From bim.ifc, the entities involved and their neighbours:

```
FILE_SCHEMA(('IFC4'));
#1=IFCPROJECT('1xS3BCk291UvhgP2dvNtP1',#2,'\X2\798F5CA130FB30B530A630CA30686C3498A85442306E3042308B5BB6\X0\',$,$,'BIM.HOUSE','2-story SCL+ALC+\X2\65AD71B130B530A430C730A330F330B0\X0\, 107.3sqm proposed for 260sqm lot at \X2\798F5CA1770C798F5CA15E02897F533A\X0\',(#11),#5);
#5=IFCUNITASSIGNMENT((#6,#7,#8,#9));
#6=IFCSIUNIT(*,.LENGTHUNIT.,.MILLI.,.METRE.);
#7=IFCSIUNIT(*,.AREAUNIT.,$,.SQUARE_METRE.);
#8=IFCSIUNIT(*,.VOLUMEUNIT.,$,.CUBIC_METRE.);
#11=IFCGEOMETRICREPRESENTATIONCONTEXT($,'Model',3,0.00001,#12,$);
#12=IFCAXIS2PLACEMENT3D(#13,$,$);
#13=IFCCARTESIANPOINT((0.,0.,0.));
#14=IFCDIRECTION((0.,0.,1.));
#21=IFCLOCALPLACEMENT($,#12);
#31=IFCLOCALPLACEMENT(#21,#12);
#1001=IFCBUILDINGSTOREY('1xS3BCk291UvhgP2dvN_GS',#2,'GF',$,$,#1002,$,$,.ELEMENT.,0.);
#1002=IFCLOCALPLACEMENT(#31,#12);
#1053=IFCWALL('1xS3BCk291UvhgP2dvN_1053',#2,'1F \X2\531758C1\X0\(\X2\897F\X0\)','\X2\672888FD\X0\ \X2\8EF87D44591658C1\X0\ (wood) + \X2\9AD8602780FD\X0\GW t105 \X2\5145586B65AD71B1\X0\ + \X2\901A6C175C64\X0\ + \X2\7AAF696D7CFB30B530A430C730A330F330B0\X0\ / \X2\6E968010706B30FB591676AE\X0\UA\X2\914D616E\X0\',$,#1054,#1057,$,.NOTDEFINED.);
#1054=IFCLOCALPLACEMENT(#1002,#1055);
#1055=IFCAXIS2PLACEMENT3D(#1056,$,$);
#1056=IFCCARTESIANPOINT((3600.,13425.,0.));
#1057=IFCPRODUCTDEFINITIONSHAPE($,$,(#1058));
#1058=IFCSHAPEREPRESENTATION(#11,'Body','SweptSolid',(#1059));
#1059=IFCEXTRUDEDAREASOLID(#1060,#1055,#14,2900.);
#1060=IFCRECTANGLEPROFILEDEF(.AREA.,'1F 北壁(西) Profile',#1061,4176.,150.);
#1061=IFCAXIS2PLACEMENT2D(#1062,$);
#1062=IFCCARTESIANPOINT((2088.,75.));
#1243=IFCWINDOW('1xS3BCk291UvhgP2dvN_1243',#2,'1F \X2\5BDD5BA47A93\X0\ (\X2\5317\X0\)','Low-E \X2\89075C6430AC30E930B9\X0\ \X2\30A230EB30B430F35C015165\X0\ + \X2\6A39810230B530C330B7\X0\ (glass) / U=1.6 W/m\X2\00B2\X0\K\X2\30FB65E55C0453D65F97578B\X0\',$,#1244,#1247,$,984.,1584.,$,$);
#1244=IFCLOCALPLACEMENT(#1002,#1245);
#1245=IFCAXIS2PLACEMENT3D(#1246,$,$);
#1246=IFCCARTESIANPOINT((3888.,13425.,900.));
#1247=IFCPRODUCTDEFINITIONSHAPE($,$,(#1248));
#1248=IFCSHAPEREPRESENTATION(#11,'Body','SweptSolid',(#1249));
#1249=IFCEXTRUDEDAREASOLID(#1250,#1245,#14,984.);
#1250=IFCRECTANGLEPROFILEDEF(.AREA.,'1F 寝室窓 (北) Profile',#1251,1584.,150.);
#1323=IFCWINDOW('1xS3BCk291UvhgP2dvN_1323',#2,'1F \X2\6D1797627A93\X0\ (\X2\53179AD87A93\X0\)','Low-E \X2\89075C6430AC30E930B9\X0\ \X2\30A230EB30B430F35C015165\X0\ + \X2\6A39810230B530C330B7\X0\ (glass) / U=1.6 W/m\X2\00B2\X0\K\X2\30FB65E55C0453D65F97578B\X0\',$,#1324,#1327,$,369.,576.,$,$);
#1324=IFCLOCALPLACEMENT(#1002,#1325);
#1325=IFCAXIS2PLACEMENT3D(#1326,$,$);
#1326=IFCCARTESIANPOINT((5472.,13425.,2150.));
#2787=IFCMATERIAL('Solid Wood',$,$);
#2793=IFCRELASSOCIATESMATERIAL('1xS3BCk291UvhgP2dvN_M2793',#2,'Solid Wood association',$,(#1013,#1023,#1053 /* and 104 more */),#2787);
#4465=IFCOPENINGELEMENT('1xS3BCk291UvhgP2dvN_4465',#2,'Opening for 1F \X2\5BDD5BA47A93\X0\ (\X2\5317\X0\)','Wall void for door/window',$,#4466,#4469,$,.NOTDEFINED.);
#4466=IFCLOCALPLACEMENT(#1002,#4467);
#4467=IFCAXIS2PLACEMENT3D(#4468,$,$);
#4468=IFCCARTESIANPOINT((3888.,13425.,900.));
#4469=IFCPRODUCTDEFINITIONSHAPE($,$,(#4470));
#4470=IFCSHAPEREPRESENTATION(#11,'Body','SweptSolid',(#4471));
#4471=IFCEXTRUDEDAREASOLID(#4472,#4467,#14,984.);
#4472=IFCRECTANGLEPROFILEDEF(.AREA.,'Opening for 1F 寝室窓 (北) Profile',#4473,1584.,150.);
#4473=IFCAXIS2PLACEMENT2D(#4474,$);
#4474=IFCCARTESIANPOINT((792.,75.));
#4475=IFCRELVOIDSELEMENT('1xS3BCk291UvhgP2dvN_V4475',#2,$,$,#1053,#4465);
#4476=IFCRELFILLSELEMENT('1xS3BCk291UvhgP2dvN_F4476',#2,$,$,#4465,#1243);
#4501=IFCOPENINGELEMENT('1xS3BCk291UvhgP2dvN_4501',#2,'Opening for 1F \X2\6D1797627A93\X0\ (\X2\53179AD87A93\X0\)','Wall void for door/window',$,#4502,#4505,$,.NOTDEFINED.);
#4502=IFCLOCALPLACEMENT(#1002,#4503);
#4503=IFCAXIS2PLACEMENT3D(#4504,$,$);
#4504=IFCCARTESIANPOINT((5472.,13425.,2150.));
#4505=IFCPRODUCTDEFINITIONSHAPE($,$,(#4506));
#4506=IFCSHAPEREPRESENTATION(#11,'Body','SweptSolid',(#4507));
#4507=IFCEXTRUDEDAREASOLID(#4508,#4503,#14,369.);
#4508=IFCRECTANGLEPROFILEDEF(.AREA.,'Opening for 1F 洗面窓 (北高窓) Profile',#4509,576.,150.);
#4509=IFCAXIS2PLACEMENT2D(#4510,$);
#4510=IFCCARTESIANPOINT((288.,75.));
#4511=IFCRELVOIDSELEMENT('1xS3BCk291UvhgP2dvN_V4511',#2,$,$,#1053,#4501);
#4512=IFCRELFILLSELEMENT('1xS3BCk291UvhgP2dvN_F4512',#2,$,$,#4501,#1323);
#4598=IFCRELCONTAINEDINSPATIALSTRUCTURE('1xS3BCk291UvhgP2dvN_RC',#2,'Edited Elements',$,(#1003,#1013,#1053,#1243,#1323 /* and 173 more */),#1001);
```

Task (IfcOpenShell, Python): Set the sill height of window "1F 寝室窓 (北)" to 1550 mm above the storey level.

```python
import numpy as np
import ifcopenshell
import ifcopenshell.api.geometry
import ifcopenshell.geom
import ifcopenshell.util.element
import ifcopenshell.util.placement
import ifcopenshell.util.shape
import ifcopenshell.util.unit

model = ifcopenshell.open("bim.ifc")
unit_scale = ifcopenshell.util.unit.calculate_unit_scale(model)

window = model.by_guid("1xS3BCk291UvhgP2dvN_1243")
opening = window.FillsVoids[0].RelatingOpeningElement
storey = ifcopenshell.util.element.get_container(window, ifc_class="IfcBuildingStorey")
level = ifcopenshell.util.placement.get_local_placement(storey.ObjectPlacement)[2, 3]

# The opening's origin need not be at the sill, so measure its lowest point.
shape = ifcopenshell.geom.create_shape(ifcopenshell.geom.settings(), opening)
bottom = ifcopenshell.util.shape.get_shape_bottom_elevation(shape, shape.geometry) / unit_scale
dz = level + 1.55 / unit_scale - bottom

shift = np.array([0.0, 0.0, dz])
# The window is not placed relative to its opening, so move both.
for product in (opening, window):
    matrix = ifcopenshell.util.placement.get_local_placement(product.ObjectPlacement)
    matrix[:3, 3] += shift
    ifcopenshell.api.geometry.edit_object_placement(model, product=product, matrix=matrix, is_si=False)

print(f"moved by {dz * unit_scale:+.3f} m")

model.write("bim_v2.ifc")
```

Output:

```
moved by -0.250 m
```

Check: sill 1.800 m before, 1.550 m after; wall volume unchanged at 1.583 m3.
